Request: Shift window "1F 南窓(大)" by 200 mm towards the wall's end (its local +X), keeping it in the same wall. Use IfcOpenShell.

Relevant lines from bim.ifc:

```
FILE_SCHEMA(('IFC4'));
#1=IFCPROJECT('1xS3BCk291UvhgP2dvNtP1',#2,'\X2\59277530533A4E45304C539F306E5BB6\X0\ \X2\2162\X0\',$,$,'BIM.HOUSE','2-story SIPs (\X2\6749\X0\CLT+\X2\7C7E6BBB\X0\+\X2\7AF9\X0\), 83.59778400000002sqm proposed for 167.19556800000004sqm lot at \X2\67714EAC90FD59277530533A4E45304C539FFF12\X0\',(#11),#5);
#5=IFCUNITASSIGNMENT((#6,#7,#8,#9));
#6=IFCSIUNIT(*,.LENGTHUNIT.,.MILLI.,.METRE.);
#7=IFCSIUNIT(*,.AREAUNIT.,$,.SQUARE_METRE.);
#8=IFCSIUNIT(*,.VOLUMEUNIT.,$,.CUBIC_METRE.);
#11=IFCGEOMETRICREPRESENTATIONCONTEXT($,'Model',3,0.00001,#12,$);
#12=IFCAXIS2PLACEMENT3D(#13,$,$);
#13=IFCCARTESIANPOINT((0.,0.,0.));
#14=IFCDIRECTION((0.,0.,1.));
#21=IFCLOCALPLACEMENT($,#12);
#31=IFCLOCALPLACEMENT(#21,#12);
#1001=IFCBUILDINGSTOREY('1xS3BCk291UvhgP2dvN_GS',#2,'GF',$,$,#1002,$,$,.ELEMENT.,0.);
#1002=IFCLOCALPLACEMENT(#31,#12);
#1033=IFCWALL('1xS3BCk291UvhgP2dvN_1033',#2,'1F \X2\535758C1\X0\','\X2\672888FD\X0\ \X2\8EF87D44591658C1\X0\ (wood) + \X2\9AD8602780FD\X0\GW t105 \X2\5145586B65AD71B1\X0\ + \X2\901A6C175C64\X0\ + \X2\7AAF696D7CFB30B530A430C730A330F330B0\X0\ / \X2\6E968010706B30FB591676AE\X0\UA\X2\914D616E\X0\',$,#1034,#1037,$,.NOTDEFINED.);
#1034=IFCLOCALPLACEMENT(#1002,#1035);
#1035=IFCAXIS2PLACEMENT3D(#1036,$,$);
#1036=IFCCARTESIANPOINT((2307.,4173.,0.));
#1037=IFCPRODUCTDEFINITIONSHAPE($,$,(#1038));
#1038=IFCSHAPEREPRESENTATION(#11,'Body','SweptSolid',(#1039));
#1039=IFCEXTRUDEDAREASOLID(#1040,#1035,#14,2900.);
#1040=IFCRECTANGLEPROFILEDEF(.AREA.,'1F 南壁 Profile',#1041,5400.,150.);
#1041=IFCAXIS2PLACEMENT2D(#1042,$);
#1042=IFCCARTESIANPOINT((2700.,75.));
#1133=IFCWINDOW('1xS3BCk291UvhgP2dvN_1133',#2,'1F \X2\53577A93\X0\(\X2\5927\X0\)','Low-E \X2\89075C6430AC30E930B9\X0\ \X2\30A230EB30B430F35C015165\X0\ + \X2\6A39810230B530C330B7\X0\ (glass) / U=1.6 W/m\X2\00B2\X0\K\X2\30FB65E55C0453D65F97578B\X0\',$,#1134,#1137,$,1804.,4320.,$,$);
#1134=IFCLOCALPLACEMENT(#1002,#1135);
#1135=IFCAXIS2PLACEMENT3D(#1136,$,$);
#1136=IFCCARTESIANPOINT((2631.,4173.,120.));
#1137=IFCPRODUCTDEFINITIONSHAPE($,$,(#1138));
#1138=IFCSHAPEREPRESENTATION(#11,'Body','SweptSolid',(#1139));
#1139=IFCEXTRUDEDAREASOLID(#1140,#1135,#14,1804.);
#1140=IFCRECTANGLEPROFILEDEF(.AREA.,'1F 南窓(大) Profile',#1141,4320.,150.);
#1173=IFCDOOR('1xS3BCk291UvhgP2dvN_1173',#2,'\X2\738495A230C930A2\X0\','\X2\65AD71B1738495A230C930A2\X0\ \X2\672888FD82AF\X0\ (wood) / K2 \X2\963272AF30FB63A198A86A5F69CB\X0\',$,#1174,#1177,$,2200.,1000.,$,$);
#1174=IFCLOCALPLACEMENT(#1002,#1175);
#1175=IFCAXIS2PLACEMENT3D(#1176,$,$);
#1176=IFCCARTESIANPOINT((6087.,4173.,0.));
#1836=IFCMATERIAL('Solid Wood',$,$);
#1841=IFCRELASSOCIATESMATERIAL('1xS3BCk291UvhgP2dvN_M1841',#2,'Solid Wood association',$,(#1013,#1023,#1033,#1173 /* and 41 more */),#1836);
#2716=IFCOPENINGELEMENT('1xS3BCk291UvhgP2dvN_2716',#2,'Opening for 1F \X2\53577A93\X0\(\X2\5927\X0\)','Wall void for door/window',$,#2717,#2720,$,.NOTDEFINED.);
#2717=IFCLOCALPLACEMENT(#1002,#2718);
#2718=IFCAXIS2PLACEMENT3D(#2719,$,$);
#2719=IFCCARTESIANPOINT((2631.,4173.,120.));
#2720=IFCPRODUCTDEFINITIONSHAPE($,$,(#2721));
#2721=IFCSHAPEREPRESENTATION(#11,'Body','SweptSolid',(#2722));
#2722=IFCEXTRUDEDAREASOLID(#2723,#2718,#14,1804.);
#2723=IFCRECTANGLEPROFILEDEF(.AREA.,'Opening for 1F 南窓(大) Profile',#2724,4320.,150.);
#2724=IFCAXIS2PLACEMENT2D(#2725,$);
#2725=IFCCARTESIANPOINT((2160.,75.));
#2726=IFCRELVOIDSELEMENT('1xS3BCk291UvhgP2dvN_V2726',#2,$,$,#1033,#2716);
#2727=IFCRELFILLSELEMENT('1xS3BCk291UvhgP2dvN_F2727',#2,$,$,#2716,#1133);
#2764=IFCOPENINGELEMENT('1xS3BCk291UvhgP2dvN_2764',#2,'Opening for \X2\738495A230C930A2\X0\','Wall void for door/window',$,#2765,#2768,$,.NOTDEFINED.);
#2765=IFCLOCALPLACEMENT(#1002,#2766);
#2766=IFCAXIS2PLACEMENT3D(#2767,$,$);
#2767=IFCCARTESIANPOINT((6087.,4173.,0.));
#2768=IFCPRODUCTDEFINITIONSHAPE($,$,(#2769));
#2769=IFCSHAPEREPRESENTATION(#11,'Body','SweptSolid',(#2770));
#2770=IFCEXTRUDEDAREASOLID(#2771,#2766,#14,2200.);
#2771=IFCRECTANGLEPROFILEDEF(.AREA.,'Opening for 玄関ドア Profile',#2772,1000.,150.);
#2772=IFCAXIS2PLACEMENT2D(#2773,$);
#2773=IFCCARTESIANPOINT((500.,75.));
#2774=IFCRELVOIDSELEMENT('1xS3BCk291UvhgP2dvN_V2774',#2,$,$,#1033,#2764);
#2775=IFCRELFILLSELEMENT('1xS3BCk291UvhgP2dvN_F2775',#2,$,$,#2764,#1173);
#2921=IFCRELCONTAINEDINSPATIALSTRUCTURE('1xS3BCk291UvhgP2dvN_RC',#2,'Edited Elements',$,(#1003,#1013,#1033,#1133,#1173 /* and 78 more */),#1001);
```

```python
import ifcopenshell
import ifcopenshell.api.geometry
import ifcopenshell.util.placement
import ifcopenshell.util.unit

model = ifcopenshell.open("bim.ifc")
unit_scale = ifcopenshell.util.unit.calculate_unit_scale(model)

window = model.by_guid("1xS3BCk291UvhgP2dvN_1133")
opening = window.FillsVoids[0].RelatingOpeningElement
wall = opening.VoidsElements[0].RelatingBuildingElement

wall_matrix = ifcopenshell.util.placement.get_local_placement(wall.ObjectPlacement)
shift = wall_matrix[:3, 0] * 0.2 / unit_scale
before = ifcopenshell.util.placement.get_local_placement(window.ObjectPlacement)[:3, 3].copy()

# The window is not placed relative to its opening, so move both.
for product in (opening, window):
    matrix = ifcopenshell.util.placement.get_local_placement(product.ObjectPlacement)
    matrix[:3, 3] += shift
    ifcopenshell.api.geometry.edit_object_placement(model, product=product, matrix=matrix, is_si=False)

after = ifcopenshell.util.placement.get_local_placement(window.ObjectPlacement)[:3, 3]
print("window moved by", (after - before).round(3) + 0.0)

model.write("bim_v2.ifc")
```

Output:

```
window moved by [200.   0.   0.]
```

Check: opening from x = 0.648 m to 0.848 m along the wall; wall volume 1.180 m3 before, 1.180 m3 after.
